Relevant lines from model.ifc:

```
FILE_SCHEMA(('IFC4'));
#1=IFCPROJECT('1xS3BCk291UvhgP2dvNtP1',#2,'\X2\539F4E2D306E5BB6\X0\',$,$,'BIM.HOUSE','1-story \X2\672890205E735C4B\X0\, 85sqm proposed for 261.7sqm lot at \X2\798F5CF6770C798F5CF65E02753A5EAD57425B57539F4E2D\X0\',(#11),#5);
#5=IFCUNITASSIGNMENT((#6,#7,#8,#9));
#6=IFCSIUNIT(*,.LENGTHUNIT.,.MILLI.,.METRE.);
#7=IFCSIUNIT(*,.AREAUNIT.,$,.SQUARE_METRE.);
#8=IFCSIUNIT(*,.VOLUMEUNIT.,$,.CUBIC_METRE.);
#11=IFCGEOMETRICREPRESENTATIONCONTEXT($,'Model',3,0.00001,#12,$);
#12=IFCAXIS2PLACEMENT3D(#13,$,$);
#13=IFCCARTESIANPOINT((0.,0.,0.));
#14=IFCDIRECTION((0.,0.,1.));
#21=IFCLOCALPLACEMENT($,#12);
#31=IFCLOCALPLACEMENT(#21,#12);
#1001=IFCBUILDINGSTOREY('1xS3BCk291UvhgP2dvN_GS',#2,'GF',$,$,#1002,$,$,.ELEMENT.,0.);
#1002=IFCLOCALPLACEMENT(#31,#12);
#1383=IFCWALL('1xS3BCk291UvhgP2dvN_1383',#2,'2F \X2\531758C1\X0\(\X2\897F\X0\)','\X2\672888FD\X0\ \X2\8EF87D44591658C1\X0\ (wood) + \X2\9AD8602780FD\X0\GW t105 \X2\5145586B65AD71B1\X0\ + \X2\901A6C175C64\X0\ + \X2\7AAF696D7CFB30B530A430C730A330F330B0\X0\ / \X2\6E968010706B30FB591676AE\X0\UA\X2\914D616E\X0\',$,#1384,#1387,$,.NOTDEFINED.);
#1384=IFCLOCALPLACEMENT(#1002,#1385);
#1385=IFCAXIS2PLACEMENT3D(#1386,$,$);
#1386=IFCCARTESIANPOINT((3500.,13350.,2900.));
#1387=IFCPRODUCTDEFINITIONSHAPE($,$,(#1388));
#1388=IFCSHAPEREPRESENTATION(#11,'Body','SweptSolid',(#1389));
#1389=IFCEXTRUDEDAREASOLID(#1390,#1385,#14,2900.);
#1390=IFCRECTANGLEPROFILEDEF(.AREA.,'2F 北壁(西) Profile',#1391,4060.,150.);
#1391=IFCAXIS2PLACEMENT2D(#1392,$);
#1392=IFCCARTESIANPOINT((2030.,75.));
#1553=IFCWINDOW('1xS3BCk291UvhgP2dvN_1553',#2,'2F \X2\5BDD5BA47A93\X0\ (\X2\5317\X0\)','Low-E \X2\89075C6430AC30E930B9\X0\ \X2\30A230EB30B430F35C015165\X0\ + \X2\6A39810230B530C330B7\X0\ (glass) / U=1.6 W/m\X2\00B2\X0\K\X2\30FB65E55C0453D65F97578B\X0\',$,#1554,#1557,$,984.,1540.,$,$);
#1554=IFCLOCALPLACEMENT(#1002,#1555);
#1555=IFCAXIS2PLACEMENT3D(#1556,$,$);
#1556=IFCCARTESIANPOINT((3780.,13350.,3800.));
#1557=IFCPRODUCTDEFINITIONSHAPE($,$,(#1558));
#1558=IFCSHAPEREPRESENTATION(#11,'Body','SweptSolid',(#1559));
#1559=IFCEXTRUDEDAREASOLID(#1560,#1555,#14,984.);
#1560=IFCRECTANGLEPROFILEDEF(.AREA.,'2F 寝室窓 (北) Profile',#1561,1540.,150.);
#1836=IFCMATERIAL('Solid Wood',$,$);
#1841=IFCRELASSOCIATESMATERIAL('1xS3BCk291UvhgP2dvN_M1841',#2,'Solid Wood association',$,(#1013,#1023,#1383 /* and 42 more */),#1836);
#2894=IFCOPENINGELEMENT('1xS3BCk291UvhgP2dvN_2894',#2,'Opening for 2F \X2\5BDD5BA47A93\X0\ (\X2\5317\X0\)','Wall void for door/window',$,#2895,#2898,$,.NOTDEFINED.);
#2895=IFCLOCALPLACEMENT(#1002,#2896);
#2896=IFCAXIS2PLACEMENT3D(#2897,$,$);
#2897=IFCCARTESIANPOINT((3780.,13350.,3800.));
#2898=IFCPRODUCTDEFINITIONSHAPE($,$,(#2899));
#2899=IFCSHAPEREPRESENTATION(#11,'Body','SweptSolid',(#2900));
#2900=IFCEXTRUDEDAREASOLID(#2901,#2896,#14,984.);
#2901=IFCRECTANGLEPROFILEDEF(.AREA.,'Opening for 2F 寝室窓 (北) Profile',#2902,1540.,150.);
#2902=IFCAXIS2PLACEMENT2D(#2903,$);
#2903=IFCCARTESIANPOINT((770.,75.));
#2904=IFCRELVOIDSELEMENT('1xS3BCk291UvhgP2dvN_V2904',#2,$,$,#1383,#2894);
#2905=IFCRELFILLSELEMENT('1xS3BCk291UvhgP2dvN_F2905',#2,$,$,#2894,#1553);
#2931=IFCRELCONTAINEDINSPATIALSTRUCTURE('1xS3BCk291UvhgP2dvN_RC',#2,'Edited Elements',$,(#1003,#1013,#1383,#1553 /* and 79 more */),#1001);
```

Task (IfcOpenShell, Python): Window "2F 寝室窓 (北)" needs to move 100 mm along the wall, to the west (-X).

```python
import ifcopenshell
import ifcopenshell.api.geometry
import ifcopenshell.util.placement
import ifcopenshell.util.unit

model = ifcopenshell.open("model.ifc")
unit_scale = ifcopenshell.util.unit.calculate_unit_scale(model)

window = model.by_guid("1xS3BCk291UvhgP2dvN_1553")
opening = window.FillsVoids[0].RelatingOpeningElement
wall = opening.VoidsElements[0].RelatingBuildingElement

wall_matrix = ifcopenshell.util.placement.get_local_placement(wall.ObjectPlacement)
shift = wall_matrix[:3, 0] * -0.1 / unit_scale
before = ifcopenshell.util.placement.get_local_placement(window.ObjectPlacement)[:3, 3].copy()

# The window is not placed relative to its opening, so move both.
for product in (opening, window):
    matrix = ifcopenshell.util.placement.get_local_placement(product.ObjectPlacement)
    matrix[:3, 3] += shift
    ifcopenshell.api.geometry.edit_object_placement(model, product=product, matrix=matrix, is_si=False)

after = ifcopenshell.util.placement.get_local_placement(window.ObjectPlacement)[:3, 3]
print("window moved by", (after - before).round(3) + 0.0)

model.write("model_edited.ifc")
```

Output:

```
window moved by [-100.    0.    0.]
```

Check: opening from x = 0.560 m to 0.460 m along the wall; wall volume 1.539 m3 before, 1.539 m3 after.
